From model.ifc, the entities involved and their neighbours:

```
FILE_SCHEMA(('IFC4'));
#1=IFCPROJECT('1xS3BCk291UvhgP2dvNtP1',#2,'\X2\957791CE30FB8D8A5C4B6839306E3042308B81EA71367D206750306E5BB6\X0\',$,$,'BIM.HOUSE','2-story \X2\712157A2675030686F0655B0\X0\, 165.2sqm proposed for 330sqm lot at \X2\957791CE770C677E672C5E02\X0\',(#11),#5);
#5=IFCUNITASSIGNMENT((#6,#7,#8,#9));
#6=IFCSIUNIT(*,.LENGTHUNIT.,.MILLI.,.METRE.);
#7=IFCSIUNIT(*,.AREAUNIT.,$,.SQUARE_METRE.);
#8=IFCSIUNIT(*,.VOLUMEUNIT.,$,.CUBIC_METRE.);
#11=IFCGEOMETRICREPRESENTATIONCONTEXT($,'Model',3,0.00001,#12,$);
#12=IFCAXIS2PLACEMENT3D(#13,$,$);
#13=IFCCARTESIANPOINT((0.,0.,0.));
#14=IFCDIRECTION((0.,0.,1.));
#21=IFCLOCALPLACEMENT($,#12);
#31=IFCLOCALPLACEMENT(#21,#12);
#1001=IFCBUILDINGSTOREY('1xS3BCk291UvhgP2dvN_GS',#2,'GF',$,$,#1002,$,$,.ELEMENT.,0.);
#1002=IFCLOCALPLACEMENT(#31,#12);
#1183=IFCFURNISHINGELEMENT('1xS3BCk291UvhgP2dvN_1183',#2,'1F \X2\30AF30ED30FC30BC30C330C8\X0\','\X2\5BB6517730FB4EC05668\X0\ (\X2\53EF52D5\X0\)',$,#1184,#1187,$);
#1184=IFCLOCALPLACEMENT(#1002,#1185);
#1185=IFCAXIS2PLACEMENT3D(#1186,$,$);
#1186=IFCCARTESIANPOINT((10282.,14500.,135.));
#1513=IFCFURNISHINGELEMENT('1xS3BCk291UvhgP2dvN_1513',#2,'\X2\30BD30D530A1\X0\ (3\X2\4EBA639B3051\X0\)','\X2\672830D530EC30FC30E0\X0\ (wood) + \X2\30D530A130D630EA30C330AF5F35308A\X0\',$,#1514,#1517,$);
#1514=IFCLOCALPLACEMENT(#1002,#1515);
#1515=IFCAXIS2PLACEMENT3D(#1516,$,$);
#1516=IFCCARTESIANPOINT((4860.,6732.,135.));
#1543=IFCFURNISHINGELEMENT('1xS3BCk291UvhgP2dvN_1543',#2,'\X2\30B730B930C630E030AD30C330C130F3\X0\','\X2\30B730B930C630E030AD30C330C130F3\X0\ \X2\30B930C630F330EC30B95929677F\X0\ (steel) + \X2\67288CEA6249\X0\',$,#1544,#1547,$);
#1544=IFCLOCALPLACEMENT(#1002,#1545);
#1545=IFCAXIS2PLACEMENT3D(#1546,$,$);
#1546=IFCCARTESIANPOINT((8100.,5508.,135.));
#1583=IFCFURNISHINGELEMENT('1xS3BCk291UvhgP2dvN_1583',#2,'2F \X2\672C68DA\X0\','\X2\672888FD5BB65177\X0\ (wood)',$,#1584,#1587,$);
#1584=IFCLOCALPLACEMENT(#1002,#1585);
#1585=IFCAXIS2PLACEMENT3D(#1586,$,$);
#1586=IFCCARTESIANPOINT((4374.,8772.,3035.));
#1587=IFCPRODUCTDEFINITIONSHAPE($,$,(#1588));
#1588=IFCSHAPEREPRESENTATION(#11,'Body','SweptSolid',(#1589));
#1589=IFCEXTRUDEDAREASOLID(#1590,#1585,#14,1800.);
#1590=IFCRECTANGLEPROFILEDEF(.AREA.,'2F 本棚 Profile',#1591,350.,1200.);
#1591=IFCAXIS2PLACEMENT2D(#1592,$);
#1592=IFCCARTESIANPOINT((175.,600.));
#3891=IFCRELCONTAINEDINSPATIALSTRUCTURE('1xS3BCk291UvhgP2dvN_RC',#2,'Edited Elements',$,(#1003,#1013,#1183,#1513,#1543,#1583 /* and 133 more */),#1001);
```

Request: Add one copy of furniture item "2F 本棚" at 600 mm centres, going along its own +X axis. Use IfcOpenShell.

```python
import ifcopenshell
import ifcopenshell.api.geometry
import ifcopenshell.api.root
import ifcopenshell.util.element
import ifcopenshell.util.placement

model = ifcopenshell.open("model.ifc")


def reuse_history(source, copy):
    """copy_class also copies each property set's owner history, people and application; keep the originals."""
    for rel in copy.IsDefinedBy:
        if rel.is_a("IfcRelDefinesByProperties") and (history := rel.RelatingPropertyDefinition.OwnerHistory):
            rel.RelatingPropertyDefinition.OwnerHistory = source.OwnerHistory
            ifcopenshell.util.element.remove_deep2(model, history)


source = model.by_guid("1xS3BCk291UvhgP2dvN_1583")
base = ifcopenshell.util.placement.get_local_placement(source.ObjectPlacement)
step = base[:3, 0] * 600.0

for i in range(1, 2):
    copy = ifcopenshell.api.root.copy_class(model, product=source)
    copy.Representation = ifcopenshell.util.element.copy_deep(
        model, source.Representation, exclude=["IfcGeometricRepresentationContext", "IfcRepresentationMap"]
    )
    reuse_history(source, copy)
    matrix = base.copy()
    matrix[:3, 3] += i * step
    print("added at", matrix[:3, 3].round(3) + 0.0)
    ifcopenshell.api.geometry.edit_object_placement(model, product=copy, matrix=matrix, is_si=False)

model.write("model_updated.ifc")
```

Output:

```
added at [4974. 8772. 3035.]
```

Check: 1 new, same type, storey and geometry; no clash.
